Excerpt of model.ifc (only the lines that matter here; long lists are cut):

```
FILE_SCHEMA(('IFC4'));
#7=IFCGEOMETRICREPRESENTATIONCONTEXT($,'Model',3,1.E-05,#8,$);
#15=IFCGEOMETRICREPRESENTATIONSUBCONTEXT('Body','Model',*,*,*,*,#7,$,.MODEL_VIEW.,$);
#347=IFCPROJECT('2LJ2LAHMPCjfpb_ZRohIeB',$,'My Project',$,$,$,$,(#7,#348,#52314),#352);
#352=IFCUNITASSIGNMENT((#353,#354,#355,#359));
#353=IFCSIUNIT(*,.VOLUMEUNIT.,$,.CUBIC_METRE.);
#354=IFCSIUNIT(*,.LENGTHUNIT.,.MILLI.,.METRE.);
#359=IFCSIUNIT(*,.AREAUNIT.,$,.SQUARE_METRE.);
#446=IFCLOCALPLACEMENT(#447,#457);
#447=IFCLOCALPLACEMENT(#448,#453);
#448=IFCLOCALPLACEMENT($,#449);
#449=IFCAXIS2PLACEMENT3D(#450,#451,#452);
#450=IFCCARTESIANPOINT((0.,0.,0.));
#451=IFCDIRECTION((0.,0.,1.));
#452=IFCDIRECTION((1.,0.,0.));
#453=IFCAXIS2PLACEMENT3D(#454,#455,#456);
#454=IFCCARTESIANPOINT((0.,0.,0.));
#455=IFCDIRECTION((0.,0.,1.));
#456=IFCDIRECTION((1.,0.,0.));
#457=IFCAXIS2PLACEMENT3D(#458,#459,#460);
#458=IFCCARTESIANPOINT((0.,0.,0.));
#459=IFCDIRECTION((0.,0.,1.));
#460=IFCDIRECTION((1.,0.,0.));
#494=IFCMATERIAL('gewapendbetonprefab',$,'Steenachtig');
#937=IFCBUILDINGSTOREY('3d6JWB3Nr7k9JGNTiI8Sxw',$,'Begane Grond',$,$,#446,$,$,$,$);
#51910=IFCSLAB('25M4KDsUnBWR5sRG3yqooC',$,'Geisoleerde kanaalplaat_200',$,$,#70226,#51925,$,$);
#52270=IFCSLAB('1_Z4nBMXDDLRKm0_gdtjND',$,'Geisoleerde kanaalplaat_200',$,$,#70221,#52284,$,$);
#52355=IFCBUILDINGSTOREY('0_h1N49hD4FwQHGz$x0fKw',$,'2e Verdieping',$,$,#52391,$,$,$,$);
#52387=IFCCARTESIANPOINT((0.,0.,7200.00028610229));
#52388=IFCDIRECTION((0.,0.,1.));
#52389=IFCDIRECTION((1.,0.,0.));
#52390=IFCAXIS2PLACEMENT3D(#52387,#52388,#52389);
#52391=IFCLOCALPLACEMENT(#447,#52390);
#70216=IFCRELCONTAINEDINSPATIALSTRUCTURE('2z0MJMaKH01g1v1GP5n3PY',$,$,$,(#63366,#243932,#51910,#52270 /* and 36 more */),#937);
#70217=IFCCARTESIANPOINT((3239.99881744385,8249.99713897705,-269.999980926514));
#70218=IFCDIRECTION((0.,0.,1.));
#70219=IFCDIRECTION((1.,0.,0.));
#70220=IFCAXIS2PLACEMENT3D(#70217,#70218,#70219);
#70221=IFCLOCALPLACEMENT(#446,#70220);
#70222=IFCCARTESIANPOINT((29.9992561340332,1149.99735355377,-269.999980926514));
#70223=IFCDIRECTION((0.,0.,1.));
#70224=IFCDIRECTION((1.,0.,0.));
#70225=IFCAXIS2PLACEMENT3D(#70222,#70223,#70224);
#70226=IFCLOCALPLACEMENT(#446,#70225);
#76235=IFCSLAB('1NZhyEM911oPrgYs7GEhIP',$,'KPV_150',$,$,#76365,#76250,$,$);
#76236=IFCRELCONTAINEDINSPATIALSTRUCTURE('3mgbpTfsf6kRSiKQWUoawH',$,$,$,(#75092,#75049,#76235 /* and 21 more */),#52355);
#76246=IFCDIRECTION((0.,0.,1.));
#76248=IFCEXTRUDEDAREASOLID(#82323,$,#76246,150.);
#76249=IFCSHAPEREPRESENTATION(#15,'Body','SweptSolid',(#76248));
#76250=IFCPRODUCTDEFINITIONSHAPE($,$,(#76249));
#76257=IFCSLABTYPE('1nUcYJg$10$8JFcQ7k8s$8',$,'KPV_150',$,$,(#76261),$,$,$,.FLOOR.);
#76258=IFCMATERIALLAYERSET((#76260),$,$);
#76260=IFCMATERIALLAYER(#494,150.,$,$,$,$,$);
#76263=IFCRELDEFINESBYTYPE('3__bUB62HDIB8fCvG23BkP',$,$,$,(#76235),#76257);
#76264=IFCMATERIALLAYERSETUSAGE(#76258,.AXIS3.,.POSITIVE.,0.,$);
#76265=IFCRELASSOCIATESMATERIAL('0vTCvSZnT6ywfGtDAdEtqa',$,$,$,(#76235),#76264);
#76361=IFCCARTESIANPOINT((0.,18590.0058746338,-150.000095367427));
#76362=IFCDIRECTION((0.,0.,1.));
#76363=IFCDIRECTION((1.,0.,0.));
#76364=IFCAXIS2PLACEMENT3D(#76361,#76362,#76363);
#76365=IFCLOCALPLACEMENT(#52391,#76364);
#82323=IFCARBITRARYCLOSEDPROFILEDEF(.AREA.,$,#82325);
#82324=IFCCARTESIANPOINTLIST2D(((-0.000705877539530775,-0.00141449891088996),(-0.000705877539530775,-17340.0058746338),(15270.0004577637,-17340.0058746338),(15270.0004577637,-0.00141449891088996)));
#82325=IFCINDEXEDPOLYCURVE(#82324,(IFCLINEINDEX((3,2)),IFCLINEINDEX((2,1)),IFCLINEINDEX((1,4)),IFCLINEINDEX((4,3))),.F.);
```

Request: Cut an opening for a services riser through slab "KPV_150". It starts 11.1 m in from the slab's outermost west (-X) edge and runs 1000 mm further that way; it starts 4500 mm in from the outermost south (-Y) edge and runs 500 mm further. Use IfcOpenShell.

```python
import numpy as np
import ifcopenshell
import ifcopenshell.api.feature
import ifcopenshell.api.geometry
import ifcopenshell.api.root
import ifcopenshell.geom
import ifcopenshell.util.placement
import ifcopenshell.util.representation
import ifcopenshell.util.shape
import ifcopenshell.util.unit

model = ifcopenshell.open("model.ifc")
unit_scale = ifcopenshell.util.unit.calculate_unit_scale(model)
settings = ifcopenshell.geom.settings()


def volume(element):
    """Net volume in cubic metres, openings subtracted."""
    shape = ifcopenshell.geom.create_shape(settings, element)
    return ifcopenshell.util.shape.get_volume(shape.geometry)


slab = model.by_guid("1NZhyEM911oPrgYs7GEhIP")
before = volume(slab)

# Extent in the slab's own axes, in metres. The edges named are its -X and -Y sides.
slab_shape = ifcopenshell.geom.create_shape(settings, slab)
vertices = ifcopenshell.util.shape.get_vertices(slab_shape.geometry)
x_min, y_min, bottom = vertices.min(axis=0)
top = vertices[:, 2].max()

opening = ifcopenshell.api.root.create_entity(model, ifc_class="IfcOpeningElement", name="Services riser opening", predefined_type="OPENING")
context = ifcopenshell.util.representation.get_context(model, "Model", "Body", "MODEL_VIEW")
width, depth = 1, 0.5
outline = [(0.0, 0.0), (width, 0.0), (width, depth), (0.0, depth), (0.0, 0.0)]
# Overshoot both faces by 50 mm so the cut is clean.
shape = ifcopenshell.api.geometry.add_slab_representation(
    model, context=context, depth=top - bottom + 0.1, polyline=outline
)
ifcopenshell.api.geometry.assign_representation(model, product=opening, representation=shape)

matrix = ifcopenshell.util.placement.get_local_placement(slab.ObjectPlacement)
matrix[:, 3] = matrix @ np.append(np.array([x_min + 11.1, y_min + 4.5, bottom - 0.05]) / unit_scale, 1.0)
ifcopenshell.api.geometry.edit_object_placement(model, product=opening, matrix=matrix, is_si=False)
ifcopenshell.api.feature.add_feature(model, feature=opening, element=slab)

after = volume(slab)

print(f"slab volume {before:.3f} -> {after:.3f} m3")

model.write("model_updated.ifc")
```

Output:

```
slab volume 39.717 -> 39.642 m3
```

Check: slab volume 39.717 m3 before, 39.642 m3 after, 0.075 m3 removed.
